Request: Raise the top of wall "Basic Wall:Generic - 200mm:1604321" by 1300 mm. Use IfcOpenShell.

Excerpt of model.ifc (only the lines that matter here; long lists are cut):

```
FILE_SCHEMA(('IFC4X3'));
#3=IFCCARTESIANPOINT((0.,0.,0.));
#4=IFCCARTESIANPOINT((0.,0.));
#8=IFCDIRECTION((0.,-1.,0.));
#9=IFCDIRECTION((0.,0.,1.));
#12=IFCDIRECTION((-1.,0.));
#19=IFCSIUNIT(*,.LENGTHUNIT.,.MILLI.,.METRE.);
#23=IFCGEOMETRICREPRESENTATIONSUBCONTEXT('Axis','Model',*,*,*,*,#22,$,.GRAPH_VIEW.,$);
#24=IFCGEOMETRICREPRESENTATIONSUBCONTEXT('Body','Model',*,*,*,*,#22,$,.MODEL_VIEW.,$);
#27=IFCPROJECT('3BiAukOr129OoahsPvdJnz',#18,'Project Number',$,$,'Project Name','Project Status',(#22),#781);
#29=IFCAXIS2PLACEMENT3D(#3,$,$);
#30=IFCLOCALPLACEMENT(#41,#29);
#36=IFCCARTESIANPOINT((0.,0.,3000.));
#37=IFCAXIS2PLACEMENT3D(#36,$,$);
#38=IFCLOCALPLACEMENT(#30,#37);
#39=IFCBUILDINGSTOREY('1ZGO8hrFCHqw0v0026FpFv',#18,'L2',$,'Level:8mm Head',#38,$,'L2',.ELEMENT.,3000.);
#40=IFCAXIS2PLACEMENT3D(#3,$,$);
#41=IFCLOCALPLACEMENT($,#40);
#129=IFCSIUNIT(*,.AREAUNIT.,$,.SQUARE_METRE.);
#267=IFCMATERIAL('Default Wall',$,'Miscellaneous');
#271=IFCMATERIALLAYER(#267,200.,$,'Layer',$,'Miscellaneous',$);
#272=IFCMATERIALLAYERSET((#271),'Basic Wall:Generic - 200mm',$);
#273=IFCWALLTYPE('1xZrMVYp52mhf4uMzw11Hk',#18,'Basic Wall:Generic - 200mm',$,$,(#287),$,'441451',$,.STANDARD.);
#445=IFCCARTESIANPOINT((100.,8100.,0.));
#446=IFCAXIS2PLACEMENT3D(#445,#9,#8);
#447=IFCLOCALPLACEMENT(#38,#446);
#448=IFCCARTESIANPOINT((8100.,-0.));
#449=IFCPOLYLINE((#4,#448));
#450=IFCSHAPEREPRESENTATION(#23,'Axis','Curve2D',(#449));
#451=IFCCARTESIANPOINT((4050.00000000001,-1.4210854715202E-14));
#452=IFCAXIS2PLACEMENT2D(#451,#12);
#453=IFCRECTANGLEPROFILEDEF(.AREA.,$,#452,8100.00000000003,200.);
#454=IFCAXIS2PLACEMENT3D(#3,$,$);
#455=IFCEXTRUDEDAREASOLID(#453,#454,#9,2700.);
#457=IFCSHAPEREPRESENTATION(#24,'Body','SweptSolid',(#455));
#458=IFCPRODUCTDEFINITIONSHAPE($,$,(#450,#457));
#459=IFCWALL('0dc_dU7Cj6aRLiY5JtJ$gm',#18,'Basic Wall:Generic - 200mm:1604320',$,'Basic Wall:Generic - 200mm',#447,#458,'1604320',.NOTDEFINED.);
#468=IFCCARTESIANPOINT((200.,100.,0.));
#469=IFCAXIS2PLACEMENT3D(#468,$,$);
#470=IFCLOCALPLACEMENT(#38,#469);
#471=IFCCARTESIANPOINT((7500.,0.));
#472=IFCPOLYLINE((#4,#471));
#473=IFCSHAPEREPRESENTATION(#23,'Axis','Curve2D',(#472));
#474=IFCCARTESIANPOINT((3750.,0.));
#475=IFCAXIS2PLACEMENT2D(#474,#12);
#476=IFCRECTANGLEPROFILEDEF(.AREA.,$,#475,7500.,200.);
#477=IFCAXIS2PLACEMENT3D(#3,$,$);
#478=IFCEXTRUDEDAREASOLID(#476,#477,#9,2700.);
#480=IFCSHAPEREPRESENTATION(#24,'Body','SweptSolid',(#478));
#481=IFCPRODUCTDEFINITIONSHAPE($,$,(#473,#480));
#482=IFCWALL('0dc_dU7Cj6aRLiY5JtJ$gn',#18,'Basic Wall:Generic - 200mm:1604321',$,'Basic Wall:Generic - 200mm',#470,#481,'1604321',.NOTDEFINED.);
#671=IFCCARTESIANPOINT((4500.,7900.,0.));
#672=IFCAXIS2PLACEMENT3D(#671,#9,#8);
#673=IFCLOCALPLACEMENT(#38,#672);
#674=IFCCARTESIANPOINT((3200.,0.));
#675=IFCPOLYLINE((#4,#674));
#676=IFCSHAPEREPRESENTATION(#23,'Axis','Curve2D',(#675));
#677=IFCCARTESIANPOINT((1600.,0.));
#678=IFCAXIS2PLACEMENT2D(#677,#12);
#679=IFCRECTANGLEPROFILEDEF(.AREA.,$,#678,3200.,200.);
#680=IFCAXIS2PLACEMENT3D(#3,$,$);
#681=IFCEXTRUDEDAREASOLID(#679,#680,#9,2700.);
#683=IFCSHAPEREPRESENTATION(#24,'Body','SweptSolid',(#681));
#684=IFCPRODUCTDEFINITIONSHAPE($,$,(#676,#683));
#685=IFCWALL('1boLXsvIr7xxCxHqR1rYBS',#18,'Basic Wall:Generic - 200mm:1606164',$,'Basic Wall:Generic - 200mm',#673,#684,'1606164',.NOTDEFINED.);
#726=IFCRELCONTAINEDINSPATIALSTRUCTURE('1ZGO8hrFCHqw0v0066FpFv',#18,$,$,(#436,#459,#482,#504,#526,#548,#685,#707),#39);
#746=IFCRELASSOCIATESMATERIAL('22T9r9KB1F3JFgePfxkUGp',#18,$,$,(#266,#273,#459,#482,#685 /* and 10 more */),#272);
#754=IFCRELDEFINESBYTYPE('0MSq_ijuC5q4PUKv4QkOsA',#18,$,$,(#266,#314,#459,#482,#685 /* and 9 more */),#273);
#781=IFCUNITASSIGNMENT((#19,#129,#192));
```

```python
import ifcopenshell
import ifcopenshell.geom
import ifcopenshell.util.representation
import ifcopenshell.util.shape
import ifcopenshell.util.unit

model = ifcopenshell.open("model.ifc")
unit_scale = ifcopenshell.util.unit.calculate_unit_scale(model)
settings = ifcopenshell.geom.settings()


def volume(element):
    """Net volume in cubic metres, openings subtracted."""
    shape = ifcopenshell.geom.create_shape(settings, element)
    return ifcopenshell.util.shape.get_volume(shape.geometry)


wall = model.by_id(482)
before = volume(wall)

body = ifcopenshell.util.representation.get_representation(wall, "Model", "Body")
solid = body.Items[0]
old_height = solid.Depth
solid.Depth += 1.3 / unit_scale
after = volume(wall)

print(f"height {old_height:g} -> {solid.Depth:g}, volume {before:.3f} -> {after:.3f} m3")

model.write("model-out.ifc")
```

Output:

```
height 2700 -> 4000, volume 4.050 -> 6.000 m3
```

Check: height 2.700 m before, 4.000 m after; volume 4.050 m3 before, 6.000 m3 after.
